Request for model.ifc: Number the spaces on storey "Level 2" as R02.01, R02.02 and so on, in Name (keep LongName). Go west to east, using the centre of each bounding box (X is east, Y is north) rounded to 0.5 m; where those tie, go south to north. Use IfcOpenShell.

First a look at what the model holds.

```python
import ifcopenshell
import ifcopenshell.util.element
import ifcopenshell.util.placement

model = ifcopenshell.open("model.ifc")
print(model.schema)
storey = next(s for s in model.by_type("IfcBuildingStorey") if s.Name == "Level 2")
spaces = [e for e in ifcopenshell.util.element.get_decomposition(storey) if e.is_a("IfcSpace")]
for e in sorted(spaces, key=lambda e: e.id()):
    origin = ifcopenshell.util.placement.get_local_placement(e.ObjectPlacement)[:3, 3]
    print(e.id(), e.Name, e.LongName, origin.round(2) + 0.0, sep=" | ")
```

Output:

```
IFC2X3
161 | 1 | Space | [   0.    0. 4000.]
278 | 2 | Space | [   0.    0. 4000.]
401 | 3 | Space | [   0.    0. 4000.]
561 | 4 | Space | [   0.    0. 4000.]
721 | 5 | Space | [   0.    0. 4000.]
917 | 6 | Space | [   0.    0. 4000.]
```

```python
import ifcopenshell
import ifcopenshell.geom
import ifcopenshell.util.element
import ifcopenshell.util.shape

model = ifcopenshell.open("model.ifc")
settings = ifcopenshell.geom.settings()
settings.set("use-world-coords", True)


def centre(element):
    shape = ifcopenshell.geom.create_shape(settings, element)
    return ifcopenshell.util.shape.get_bbox_centroid(shape.geometry)


storey = next(s for s in model.by_type("IfcBuildingStorey") if s.Name == "Level 2")
spaces = [e for e in ifcopenshell.util.element.get_decomposition(storey) if e.is_a("IfcSpace")]

# Insertion points can sit at a corner or the storey origin, so sort by the geometry (in metres).
centres = {e: centre(e) for e in spaces}
spaces.sort(key=lambda e: (round(centres[e][0] / 0.5), centres[e][1]))

for i, e in enumerate(spaces, start=1):
    number = f"R02.{i:02d}"
    e.Name = number
    print(e.id(), number)

model.write("model-out.ifc")
```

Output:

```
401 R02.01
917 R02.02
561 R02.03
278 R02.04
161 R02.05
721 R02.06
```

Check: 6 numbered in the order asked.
